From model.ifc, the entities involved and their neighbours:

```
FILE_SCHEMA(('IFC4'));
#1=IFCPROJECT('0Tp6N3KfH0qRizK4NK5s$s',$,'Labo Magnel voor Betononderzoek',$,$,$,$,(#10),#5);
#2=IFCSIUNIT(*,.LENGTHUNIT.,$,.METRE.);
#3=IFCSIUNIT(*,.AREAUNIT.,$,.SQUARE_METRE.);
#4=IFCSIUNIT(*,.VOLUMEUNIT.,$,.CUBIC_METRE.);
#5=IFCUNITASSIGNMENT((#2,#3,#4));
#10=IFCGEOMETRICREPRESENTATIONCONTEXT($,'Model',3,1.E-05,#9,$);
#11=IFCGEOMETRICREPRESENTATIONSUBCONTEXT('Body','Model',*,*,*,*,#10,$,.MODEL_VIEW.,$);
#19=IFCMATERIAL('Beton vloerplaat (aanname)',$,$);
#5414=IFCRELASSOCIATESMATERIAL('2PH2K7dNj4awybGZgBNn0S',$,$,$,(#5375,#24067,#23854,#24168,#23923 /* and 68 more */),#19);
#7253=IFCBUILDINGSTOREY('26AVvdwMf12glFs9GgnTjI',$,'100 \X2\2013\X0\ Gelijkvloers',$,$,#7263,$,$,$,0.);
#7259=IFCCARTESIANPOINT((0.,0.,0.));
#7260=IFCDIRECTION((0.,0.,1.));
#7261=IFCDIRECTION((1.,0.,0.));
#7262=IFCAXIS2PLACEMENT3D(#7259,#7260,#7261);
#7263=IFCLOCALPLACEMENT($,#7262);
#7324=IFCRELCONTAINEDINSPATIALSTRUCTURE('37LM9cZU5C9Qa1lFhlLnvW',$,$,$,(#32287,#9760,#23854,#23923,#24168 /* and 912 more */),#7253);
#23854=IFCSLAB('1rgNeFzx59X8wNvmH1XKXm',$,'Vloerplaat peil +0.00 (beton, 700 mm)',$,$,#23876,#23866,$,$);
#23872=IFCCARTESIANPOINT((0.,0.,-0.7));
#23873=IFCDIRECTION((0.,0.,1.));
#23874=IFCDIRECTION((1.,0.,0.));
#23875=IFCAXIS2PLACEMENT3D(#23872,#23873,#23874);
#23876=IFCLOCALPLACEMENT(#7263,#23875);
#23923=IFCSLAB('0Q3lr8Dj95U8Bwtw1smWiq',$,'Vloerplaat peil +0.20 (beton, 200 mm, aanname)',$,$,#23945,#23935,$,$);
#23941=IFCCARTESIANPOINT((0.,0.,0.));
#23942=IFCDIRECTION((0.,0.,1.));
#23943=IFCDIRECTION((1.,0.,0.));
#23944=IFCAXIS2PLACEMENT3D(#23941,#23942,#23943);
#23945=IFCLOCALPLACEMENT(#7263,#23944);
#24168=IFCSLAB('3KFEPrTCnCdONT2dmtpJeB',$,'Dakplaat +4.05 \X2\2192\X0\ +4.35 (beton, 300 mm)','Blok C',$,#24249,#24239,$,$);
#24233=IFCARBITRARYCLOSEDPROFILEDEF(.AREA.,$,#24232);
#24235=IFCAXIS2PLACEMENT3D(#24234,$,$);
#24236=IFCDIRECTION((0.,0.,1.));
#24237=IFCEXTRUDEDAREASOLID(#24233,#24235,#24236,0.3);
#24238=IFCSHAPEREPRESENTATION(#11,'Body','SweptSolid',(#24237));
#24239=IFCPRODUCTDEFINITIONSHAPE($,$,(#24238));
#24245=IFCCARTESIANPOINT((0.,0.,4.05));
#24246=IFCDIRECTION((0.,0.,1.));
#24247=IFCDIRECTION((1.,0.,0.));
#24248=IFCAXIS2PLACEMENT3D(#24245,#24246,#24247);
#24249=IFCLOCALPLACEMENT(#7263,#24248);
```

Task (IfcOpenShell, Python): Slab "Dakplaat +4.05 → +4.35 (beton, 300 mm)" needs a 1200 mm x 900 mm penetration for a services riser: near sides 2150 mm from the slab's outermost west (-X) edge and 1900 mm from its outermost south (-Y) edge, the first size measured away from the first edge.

```python
import numpy as np
import ifcopenshell
import ifcopenshell.api.feature
import ifcopenshell.api.geometry
import ifcopenshell.api.root
import ifcopenshell.geom
import ifcopenshell.util.placement
import ifcopenshell.util.representation
import ifcopenshell.util.shape
import ifcopenshell.util.unit

model = ifcopenshell.open("model.ifc")
unit_scale = ifcopenshell.util.unit.calculate_unit_scale(model)
settings = ifcopenshell.geom.settings()


def volume(element):
    """Net volume in cubic metres, openings subtracted."""
    shape = ifcopenshell.geom.create_shape(settings, element)
    return ifcopenshell.util.shape.get_volume(shape.geometry)


slab = model.by_guid("3KFEPrTCnCdONT2dmtpJeB")
before = volume(slab)

# Extent in the slab's own axes, in metres. The edges named are its -X and -Y sides.
slab_shape = ifcopenshell.geom.create_shape(settings, slab)
vertices = ifcopenshell.util.shape.get_vertices(slab_shape.geometry)
x_min, y_min, bottom = vertices.min(axis=0)
top = vertices[:, 2].max()

opening = ifcopenshell.api.root.create_entity(model, ifc_class="IfcOpeningElement", name="Services riser opening", predefined_type="OPENING")
context = ifcopenshell.util.representation.get_context(model, "Model", "Body", "MODEL_VIEW")
width, depth = 1.2, 0.9
outline = [(0.0, 0.0), (width, 0.0), (width, depth), (0.0, depth), (0.0, 0.0)]
# Overshoot both faces by 50 mm so the cut is clean.
shape = ifcopenshell.api.geometry.add_slab_representation(
    model, context=context, depth=top - bottom + 0.1, polyline=outline
)
ifcopenshell.api.geometry.assign_representation(model, product=opening, representation=shape)

matrix = ifcopenshell.util.placement.get_local_placement(slab.ObjectPlacement)
matrix[:, 3] = matrix @ np.append(np.array([x_min + 2.15, y_min + 1.9, bottom - 0.05]) / unit_scale, 1.0)
ifcopenshell.api.geometry.edit_object_placement(model, product=opening, matrix=matrix, is_si=False)
ifcopenshell.api.feature.add_feature(model, feature=opening, element=slab)

after = volume(slab)

print(f"slab volume {before:.3f} -> {after:.3f} m3")

model.write("model_v2.ifc")
```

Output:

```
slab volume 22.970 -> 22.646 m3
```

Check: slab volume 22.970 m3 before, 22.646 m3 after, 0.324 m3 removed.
